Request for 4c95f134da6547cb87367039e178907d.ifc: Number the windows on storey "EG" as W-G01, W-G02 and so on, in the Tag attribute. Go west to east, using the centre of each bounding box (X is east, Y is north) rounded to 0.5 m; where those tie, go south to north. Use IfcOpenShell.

First a look at what the model holds.

```python
import ifcopenshell
import ifcopenshell.util.element
import ifcopenshell.util.placement

model = ifcopenshell.open("4c95f134da6547cb87367039e178907d.ifc")
print(model.schema)
storey = next(s for s in model.by_type("IfcBuildingStorey") if s.Name == "EG")
windows = [e for e in ifcopenshell.util.element.get_decomposition(storey) if e.is_a("IfcWindow")]
for e in sorted(windows, key=lambda e: e.id()):
    origin = ifcopenshell.util.placement.get_local_placement(e.ObjectPlacement)[:3, 3]
    print(e.id(), e.Tag, e.Name, origin.round(2) + 0.0, sep=" | ")
```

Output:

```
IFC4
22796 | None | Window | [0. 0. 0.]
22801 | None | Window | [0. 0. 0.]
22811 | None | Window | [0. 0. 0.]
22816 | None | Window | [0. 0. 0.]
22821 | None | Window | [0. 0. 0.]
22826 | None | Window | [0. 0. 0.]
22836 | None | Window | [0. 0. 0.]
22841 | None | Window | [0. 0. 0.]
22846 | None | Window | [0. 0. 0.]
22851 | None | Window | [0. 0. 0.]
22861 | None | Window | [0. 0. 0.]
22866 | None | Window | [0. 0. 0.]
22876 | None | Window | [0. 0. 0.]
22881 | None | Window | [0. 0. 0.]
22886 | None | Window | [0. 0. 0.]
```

```python
import ifcopenshell
import ifcopenshell.geom
import ifcopenshell.util.element
import ifcopenshell.util.shape

model = ifcopenshell.open("4c95f134da6547cb87367039e178907d.ifc")
settings = ifcopenshell.geom.settings()
settings.set("use-world-coords", True)


def centre(element):
    shape = ifcopenshell.geom.create_shape(settings, element)
    return ifcopenshell.util.shape.get_bbox_centroid(shape.geometry)


storey = next(s for s in model.by_type("IfcBuildingStorey") if s.Name == "EG")
windows = [e for e in ifcopenshell.util.element.get_decomposition(storey) if e.is_a("IfcWindow")]

# Insertion points can sit at a corner or the storey origin, so sort by the geometry (in metres).
centres = {e: centre(e) for e in windows}
windows.sort(key=lambda e: (round(centres[e][0] / 0.5), centres[e][1]))

for i, e in enumerate(windows, start=1):
    number = f"W-G{i:02d}"
    e.Tag = number
    print(e.id(), number)

model.write("4c95f134da6547cb87367039e178907d_v2.ifc")
```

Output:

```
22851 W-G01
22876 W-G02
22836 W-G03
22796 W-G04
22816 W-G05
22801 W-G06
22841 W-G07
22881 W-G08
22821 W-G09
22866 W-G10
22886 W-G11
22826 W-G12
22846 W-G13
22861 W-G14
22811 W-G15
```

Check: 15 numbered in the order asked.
